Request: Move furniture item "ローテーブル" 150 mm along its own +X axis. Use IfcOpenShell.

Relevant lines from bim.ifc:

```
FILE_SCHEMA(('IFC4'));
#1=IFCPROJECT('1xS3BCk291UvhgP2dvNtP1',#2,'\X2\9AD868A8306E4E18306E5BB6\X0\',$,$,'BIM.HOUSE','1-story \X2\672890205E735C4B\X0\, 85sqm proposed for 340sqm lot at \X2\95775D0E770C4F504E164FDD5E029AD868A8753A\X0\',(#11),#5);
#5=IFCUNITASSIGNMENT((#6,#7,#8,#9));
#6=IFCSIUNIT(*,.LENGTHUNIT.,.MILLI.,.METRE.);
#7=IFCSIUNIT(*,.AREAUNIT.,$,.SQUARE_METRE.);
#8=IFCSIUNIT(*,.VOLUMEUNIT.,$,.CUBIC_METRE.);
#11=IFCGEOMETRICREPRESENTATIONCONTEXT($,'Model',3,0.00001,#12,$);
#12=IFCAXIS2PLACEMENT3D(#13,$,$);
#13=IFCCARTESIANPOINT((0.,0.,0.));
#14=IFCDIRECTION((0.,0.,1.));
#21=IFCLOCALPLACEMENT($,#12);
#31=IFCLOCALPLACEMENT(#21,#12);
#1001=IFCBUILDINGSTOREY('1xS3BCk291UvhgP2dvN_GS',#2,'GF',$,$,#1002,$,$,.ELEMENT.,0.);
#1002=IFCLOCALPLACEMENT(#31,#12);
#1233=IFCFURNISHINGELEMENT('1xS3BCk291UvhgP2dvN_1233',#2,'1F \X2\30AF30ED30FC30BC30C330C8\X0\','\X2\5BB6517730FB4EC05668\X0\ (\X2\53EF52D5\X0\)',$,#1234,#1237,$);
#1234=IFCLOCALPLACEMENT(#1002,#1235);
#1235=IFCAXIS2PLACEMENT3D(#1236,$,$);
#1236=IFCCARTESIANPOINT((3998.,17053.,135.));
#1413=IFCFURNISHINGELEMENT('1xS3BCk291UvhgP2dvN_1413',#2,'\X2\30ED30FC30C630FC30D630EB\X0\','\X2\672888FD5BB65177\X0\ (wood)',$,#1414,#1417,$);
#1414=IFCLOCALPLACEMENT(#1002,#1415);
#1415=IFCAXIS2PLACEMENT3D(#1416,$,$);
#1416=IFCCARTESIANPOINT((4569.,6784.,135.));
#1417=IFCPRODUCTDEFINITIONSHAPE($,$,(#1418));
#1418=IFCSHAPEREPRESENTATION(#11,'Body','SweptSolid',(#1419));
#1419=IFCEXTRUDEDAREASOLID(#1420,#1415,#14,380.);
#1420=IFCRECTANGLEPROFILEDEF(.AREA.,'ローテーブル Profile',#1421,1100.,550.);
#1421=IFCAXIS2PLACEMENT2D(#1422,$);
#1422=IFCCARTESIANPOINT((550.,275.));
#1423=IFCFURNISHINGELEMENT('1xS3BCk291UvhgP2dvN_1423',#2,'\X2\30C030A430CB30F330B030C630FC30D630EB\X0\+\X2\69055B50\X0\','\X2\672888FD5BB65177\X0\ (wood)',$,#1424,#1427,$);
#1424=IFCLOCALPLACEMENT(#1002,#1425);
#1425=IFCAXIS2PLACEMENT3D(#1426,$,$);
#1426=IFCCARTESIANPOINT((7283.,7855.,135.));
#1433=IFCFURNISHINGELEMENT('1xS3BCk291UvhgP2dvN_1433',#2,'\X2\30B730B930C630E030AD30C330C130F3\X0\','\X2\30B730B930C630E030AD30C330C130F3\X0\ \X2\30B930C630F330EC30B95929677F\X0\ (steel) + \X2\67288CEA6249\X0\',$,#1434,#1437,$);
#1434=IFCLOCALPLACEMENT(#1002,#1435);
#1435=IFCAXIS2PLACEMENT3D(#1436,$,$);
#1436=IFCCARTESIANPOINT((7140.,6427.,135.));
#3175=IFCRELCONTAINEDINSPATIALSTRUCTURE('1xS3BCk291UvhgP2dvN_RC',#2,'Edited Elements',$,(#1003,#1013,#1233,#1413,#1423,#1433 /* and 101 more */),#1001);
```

```python
import ifcopenshell
import ifcopenshell.api.geometry
import ifcopenshell.util.placement
import ifcopenshell.util.unit

model = ifcopenshell.open("bim.ifc")
unit_scale = ifcopenshell.util.unit.calculate_unit_scale(model)

item = model.by_guid("1xS3BCk291UvhgP2dvN_1413")
matrix = ifcopenshell.util.placement.get_local_placement(item.ObjectPlacement)
matrix[:3, 3] += matrix[:3, 0] * 0.15 / unit_scale
ifcopenshell.api.geometry.edit_object_placement(model, product=item, matrix=matrix, is_si=False)

print(ifcopenshell.util.placement.get_local_placement(item.ObjectPlacement).round(3) + 0.0)

model.write("bim-out.ifc")
```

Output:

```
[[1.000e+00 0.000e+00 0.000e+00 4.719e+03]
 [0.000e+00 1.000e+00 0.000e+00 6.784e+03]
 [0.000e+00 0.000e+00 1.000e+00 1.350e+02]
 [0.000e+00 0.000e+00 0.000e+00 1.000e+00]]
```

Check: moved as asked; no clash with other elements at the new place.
